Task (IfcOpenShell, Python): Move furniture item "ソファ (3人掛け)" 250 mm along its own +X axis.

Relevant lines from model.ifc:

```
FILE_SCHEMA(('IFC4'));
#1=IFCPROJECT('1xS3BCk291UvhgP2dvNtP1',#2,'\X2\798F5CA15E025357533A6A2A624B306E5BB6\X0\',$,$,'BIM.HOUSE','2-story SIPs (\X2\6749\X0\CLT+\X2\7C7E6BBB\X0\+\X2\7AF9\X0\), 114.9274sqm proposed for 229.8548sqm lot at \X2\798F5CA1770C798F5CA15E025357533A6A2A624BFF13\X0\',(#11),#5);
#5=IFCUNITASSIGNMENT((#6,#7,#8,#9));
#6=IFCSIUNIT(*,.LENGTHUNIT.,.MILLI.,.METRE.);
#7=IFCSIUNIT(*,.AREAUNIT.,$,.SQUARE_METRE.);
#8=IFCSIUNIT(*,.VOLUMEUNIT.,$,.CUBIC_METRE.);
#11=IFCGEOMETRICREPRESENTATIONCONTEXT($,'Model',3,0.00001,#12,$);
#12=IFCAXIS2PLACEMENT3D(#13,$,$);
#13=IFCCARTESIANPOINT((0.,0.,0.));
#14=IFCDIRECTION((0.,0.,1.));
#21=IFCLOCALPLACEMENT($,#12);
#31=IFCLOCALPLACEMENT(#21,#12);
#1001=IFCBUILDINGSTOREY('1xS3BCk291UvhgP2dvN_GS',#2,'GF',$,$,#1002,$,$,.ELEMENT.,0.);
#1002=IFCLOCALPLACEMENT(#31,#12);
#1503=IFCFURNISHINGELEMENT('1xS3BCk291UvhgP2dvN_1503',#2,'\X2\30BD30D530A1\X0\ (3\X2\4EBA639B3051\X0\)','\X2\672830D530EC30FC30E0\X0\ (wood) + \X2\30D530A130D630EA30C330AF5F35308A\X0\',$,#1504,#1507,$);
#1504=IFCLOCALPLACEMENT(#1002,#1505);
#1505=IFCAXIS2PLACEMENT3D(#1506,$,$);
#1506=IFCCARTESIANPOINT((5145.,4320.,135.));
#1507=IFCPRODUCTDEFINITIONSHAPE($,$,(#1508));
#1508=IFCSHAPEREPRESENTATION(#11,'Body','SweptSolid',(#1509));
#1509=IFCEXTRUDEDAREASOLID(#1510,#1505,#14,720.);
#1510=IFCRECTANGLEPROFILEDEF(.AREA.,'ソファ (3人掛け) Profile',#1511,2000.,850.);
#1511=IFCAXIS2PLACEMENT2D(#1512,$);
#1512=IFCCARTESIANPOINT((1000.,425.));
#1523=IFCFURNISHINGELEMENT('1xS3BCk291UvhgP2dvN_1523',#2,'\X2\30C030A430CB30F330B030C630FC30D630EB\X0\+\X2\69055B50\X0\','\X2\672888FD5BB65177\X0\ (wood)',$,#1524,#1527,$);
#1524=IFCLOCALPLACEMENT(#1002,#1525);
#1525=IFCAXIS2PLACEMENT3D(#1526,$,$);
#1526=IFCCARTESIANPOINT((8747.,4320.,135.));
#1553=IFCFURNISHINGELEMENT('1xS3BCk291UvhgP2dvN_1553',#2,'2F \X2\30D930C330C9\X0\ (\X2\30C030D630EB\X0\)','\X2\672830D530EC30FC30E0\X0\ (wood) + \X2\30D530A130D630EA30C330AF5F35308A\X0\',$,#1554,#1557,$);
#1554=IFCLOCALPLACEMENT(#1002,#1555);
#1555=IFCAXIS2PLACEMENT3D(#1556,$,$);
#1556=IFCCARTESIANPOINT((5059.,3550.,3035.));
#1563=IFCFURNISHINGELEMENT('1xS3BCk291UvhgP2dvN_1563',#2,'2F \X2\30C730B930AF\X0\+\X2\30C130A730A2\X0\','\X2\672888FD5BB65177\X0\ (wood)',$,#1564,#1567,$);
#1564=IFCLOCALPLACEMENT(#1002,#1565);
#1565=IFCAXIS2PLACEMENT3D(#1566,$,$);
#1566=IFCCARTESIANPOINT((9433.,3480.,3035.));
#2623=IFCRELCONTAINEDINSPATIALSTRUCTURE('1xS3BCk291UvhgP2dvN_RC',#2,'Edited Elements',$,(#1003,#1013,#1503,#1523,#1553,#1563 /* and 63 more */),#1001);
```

```python
import ifcopenshell
import ifcopenshell.api.geometry
import ifcopenshell.util.placement
import ifcopenshell.util.unit

model = ifcopenshell.open("model.ifc")
unit_scale = ifcopenshell.util.unit.calculate_unit_scale(model)

item = model.by_id(1503)
matrix = ifcopenshell.util.placement.get_local_placement(item.ObjectPlacement)
matrix[:3, 3] += matrix[:3, 0] * 0.25 / unit_scale
ifcopenshell.api.geometry.edit_object_placement(model, product=item, matrix=matrix, is_si=False)

print(ifcopenshell.util.placement.get_local_placement(item.ObjectPlacement).round(3) + 0.0)

model.write("model_rev.ifc")
```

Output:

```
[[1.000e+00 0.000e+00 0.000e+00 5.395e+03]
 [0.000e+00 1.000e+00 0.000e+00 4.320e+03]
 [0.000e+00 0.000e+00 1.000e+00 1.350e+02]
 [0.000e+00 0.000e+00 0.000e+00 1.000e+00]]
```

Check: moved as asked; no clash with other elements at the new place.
